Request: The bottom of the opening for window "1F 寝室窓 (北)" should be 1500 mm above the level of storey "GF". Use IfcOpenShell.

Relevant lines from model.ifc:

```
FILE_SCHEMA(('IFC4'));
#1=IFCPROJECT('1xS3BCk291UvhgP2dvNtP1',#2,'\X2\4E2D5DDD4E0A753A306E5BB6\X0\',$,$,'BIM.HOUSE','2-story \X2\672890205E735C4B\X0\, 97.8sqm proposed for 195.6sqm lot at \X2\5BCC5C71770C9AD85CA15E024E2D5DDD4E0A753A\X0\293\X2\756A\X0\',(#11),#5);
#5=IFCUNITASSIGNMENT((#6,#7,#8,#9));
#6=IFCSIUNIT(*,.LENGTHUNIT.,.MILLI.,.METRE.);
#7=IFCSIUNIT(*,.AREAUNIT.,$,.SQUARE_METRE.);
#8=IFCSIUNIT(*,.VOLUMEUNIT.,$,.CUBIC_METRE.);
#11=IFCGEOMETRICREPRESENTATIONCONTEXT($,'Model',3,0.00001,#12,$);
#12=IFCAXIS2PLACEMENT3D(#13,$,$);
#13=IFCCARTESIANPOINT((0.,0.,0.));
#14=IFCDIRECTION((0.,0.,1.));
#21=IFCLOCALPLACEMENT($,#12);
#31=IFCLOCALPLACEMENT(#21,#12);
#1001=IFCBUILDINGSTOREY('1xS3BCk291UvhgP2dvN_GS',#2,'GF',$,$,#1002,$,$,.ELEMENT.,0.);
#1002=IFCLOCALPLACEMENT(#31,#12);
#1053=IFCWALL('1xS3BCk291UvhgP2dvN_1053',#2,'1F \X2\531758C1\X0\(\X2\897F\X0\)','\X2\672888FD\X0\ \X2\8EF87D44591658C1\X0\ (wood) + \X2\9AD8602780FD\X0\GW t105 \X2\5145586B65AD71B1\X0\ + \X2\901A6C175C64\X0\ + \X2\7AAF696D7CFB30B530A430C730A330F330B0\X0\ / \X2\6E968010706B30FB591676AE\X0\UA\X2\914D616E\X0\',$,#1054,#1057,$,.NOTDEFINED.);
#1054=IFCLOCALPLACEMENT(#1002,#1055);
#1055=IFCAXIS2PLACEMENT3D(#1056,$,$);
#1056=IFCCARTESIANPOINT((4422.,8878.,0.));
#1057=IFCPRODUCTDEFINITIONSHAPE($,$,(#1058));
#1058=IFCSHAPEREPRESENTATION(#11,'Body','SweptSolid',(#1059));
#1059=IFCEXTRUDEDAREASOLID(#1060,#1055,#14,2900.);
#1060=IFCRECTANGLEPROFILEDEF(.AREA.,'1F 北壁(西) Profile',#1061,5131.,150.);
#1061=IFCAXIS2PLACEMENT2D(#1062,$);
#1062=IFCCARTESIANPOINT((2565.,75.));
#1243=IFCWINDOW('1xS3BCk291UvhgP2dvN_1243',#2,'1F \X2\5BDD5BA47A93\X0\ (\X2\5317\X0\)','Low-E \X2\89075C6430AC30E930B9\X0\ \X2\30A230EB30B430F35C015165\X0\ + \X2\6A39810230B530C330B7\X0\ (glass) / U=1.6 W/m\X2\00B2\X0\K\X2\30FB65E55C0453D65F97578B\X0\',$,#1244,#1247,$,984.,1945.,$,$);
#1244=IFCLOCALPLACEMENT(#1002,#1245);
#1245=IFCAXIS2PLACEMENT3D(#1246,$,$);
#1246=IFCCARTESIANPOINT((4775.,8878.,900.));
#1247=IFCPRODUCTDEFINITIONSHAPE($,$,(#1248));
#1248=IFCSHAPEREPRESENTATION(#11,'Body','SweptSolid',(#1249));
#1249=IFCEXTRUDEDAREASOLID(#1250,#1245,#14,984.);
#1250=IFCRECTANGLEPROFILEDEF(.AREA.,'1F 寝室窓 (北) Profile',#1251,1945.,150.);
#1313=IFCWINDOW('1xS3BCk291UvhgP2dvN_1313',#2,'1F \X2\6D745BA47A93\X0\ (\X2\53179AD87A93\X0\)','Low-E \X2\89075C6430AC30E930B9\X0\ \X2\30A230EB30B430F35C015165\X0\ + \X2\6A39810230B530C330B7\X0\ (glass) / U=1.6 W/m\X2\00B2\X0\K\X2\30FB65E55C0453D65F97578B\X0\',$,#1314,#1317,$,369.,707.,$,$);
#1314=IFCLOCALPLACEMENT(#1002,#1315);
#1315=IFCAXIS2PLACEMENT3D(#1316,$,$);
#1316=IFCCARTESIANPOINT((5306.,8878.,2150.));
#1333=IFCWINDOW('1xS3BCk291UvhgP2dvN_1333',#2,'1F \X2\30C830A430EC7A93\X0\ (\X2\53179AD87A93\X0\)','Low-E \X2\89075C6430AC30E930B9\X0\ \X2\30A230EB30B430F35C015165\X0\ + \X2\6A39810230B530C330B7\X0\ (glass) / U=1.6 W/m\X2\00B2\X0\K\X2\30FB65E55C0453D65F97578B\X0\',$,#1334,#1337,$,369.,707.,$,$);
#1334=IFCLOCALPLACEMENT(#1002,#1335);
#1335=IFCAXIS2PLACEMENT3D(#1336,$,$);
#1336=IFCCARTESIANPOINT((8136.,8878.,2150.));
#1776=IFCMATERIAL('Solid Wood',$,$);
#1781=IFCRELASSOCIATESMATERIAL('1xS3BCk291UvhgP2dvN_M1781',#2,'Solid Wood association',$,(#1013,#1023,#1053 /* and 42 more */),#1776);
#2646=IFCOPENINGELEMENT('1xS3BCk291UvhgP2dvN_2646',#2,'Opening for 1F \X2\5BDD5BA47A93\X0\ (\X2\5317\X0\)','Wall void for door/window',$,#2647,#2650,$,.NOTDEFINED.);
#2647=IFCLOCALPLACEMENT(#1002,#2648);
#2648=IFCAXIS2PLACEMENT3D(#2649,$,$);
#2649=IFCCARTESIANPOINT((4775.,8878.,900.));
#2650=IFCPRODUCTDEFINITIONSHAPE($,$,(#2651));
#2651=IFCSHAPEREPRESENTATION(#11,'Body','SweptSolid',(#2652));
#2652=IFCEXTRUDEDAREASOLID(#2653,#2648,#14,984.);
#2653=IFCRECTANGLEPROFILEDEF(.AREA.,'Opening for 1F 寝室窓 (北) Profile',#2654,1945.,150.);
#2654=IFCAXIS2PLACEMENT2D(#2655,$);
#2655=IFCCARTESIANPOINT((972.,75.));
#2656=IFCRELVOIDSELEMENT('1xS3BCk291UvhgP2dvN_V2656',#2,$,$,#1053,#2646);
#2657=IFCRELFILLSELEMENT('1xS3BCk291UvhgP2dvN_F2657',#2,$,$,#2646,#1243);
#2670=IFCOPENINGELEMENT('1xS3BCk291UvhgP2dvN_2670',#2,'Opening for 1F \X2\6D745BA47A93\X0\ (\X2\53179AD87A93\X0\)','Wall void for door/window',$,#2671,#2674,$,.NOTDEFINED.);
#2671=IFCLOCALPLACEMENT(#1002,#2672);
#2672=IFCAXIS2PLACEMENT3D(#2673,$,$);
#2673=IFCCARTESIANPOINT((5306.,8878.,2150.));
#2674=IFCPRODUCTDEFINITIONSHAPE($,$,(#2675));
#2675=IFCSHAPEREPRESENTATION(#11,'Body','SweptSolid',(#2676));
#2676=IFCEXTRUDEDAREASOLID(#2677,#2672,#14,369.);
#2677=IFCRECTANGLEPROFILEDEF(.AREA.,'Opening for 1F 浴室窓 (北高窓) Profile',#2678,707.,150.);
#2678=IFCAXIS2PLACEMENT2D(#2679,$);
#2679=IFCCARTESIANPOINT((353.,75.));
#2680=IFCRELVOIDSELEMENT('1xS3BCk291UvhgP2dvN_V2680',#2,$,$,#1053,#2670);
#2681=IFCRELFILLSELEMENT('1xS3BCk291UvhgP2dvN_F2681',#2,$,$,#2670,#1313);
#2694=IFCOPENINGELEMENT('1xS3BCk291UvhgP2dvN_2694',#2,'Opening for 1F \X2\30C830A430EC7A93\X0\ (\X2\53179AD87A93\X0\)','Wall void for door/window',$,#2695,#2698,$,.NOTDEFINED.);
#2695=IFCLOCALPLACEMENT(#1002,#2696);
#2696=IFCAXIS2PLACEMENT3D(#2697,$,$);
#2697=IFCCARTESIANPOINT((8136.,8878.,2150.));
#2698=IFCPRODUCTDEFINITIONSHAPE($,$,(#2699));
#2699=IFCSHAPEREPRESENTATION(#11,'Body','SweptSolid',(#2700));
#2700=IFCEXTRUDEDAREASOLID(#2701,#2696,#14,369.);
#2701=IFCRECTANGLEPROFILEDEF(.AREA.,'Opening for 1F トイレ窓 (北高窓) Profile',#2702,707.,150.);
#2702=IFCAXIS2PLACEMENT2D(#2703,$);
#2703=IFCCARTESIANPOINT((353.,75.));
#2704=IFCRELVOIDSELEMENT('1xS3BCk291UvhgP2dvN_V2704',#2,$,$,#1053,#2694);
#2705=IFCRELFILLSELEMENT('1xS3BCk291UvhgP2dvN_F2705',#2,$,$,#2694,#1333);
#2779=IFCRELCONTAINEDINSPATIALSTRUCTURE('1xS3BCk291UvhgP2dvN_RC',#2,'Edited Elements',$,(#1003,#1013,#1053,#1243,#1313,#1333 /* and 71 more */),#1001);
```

```python
import numpy as np
import ifcopenshell
import ifcopenshell.api.geometry
import ifcopenshell.geom
import ifcopenshell.util.element
import ifcopenshell.util.placement
import ifcopenshell.util.shape
import ifcopenshell.util.unit

model = ifcopenshell.open("model.ifc")
unit_scale = ifcopenshell.util.unit.calculate_unit_scale(model)

window = model.by_guid("1xS3BCk291UvhgP2dvN_1243")
opening = window.FillsVoids[0].RelatingOpeningElement
storey = ifcopenshell.util.element.get_container(window, ifc_class="IfcBuildingStorey")
level = ifcopenshell.util.placement.get_local_placement(storey.ObjectPlacement)[2, 3]

# The opening's origin need not be at the sill, so measure its lowest point.
shape = ifcopenshell.geom.create_shape(ifcopenshell.geom.settings(), opening)
bottom = ifcopenshell.util.shape.get_shape_bottom_elevation(shape, shape.geometry) / unit_scale
dz = level + 1.5 / unit_scale - bottom

shift = np.array([0.0, 0.0, dz])
# The window is not placed relative to its opening, so move both.
for product in (opening, window):
    matrix = ifcopenshell.util.placement.get_local_placement(product.ObjectPlacement)
    matrix[:3, 3] += shift
    ifcopenshell.api.geometry.edit_object_placement(model, product=product, matrix=matrix, is_si=False)

print(f"moved by {dz * unit_scale:+.3f} m")

model.write("model_updated.ifc")
```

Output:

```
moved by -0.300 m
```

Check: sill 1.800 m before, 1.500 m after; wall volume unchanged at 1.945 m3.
